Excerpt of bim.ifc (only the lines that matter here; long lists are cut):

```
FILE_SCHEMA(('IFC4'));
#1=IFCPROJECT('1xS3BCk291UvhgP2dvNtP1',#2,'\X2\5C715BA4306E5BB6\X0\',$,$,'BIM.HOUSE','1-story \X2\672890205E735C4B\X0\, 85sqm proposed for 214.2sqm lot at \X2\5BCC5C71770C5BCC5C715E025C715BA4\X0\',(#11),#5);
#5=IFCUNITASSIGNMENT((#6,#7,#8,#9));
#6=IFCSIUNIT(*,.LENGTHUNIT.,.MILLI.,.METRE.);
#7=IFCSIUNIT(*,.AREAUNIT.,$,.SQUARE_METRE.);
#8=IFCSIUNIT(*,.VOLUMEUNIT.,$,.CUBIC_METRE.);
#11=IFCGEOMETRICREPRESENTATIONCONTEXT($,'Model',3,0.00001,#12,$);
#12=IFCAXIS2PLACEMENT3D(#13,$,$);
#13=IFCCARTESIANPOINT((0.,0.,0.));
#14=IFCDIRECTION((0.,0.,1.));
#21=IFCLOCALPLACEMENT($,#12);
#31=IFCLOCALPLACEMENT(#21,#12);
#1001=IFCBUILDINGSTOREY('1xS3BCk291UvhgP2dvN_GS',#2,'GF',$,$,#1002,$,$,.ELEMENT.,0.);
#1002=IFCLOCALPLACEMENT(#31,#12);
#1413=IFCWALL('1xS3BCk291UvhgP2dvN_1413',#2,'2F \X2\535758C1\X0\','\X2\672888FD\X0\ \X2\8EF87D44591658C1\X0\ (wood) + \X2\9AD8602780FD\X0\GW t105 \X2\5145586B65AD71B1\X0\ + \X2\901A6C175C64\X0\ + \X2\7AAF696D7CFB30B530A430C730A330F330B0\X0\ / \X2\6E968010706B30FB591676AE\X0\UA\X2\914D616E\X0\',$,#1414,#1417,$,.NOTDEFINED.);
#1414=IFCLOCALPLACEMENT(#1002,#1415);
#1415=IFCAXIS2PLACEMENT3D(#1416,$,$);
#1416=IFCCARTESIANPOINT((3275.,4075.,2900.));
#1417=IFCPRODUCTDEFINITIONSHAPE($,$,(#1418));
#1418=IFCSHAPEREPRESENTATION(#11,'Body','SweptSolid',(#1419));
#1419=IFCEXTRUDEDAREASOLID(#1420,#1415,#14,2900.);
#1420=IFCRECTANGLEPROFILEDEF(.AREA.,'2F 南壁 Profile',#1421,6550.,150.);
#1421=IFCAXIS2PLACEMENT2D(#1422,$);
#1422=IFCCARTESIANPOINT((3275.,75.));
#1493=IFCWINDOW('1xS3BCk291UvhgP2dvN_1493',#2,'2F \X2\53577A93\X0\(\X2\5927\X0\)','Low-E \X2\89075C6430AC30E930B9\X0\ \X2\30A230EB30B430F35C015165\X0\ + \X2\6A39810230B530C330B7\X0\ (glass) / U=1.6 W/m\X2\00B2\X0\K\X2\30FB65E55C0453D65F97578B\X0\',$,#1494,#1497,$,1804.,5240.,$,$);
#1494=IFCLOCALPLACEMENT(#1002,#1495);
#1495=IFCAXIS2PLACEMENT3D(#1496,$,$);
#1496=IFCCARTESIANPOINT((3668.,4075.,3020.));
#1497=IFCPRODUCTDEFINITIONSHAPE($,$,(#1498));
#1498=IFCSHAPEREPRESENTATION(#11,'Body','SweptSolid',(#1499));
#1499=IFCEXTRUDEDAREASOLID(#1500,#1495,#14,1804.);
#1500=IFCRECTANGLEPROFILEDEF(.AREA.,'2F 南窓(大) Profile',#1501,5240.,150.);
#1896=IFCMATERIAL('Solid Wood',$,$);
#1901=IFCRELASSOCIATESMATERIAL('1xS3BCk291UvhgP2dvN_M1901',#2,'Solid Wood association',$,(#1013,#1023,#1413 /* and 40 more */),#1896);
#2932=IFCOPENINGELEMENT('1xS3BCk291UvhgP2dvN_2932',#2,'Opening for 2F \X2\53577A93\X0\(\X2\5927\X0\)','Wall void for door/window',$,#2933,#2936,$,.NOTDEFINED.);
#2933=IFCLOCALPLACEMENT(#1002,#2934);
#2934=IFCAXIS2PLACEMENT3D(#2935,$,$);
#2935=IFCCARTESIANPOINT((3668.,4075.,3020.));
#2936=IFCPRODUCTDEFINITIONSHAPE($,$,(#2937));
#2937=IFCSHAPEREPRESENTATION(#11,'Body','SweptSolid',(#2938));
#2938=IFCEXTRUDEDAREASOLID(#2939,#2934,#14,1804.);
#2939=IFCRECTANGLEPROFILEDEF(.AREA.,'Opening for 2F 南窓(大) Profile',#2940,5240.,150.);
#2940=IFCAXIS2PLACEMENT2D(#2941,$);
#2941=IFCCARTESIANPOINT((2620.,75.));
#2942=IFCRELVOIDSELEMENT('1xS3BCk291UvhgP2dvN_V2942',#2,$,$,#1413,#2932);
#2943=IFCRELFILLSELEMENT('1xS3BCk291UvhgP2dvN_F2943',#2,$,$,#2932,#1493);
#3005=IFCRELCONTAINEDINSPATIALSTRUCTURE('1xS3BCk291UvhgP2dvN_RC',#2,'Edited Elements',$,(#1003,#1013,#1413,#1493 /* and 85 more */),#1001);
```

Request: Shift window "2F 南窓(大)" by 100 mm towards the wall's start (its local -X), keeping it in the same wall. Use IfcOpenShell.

```python
import ifcopenshell
import ifcopenshell.api.geometry
import ifcopenshell.util.placement
import ifcopenshell.util.unit

model = ifcopenshell.open("bim.ifc")
unit_scale = ifcopenshell.util.unit.calculate_unit_scale(model)

window = model.by_guid("1xS3BCk291UvhgP2dvN_1493")
opening = window.FillsVoids[0].RelatingOpeningElement
wall = opening.VoidsElements[0].RelatingBuildingElement

wall_matrix = ifcopenshell.util.placement.get_local_placement(wall.ObjectPlacement)
shift = wall_matrix[:3, 0] * -0.1 / unit_scale
before = ifcopenshell.util.placement.get_local_placement(window.ObjectPlacement)[:3, 3].copy()

# The window is not placed relative to its opening, so move both.
for product in (opening, window):
    matrix = ifcopenshell.util.placement.get_local_placement(product.ObjectPlacement)
    matrix[:3, 3] += shift
    ifcopenshell.api.geometry.edit_object_placement(model, product=product, matrix=matrix, is_si=False)

after = ifcopenshell.util.placement.get_local_placement(window.ObjectPlacement)[:3, 3]
print("window moved by", (after - before).round(3) + 0.0)

model.write("bim_updated.ifc")
```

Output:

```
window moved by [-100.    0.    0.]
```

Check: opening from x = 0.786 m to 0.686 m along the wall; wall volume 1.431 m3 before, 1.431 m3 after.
